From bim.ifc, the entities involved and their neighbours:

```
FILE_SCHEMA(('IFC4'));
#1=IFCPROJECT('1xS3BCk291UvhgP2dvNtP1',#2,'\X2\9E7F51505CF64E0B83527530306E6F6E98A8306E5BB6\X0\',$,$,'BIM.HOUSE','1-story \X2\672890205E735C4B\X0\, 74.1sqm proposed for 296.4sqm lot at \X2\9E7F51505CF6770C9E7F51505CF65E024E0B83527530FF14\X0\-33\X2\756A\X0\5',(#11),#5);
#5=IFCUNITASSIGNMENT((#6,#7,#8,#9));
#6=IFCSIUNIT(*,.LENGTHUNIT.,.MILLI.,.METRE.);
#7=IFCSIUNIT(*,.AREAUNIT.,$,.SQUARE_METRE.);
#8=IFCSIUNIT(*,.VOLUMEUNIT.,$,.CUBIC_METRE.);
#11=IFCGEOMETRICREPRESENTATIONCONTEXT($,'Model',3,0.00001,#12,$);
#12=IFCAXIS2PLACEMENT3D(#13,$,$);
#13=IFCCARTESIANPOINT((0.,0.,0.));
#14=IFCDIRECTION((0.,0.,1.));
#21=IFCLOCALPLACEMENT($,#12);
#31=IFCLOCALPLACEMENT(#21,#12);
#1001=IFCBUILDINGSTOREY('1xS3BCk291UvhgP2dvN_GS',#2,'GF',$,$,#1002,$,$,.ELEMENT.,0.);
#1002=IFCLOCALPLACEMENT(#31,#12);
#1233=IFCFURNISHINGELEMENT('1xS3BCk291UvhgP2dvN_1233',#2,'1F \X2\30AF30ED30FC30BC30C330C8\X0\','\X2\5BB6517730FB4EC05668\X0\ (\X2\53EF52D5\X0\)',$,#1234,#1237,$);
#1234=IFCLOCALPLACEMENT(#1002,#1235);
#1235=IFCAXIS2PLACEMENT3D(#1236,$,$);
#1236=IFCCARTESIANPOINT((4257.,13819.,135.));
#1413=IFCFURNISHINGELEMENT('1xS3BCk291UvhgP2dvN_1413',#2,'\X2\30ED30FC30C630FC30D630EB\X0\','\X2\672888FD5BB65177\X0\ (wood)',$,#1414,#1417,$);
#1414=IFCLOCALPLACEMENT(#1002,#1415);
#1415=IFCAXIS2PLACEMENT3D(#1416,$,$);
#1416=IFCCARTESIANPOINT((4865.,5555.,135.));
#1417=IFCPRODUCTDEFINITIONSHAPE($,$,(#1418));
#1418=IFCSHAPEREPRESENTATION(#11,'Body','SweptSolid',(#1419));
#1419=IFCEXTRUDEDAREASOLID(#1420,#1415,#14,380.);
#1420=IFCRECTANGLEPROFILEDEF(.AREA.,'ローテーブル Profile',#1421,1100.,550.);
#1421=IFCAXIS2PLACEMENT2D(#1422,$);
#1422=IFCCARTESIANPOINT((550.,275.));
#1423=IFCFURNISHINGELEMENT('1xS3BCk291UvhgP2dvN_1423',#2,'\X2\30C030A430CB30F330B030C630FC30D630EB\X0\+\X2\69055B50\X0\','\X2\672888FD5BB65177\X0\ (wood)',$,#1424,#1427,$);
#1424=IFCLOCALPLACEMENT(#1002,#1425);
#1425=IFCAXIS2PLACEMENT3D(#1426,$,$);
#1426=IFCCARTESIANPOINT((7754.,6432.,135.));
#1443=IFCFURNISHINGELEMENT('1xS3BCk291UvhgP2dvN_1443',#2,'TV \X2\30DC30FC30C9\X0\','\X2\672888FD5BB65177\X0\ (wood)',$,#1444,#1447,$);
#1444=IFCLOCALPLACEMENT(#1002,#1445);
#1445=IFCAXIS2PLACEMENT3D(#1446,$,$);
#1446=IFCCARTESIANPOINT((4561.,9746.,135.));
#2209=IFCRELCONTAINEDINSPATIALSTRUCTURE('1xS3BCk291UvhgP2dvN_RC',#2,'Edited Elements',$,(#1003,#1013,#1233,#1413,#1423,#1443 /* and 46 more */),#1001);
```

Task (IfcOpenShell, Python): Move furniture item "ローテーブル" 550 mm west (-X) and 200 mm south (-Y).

```python
import ifcopenshell
import ifcopenshell.api.geometry
import ifcopenshell.util.placement

model = ifcopenshell.open("bim.ifc")

item = model.by_id(1413)
matrix = ifcopenshell.util.placement.get_local_placement(item.ObjectPlacement)
matrix[0, 3] -= 550.0
matrix[1, 3] -= 200.0
ifcopenshell.api.geometry.edit_object_placement(model, product=item, matrix=matrix, is_si=False)

print(ifcopenshell.util.placement.get_local_placement(item.ObjectPlacement).round(3) + 0.0)

model.write("bim_v2.ifc")
```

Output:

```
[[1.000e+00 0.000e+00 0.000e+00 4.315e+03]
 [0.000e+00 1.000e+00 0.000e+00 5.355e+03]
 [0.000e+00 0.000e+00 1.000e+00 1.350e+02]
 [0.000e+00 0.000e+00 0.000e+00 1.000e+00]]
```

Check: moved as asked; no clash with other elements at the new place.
